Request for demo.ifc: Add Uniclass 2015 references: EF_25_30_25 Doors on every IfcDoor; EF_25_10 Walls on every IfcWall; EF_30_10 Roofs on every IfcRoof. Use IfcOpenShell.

First a look at what the model holds.

```python
import ifcopenshell

model = ifcopenshell.open("demo.ifc")
print(model.schema)
print("classifications:", [c.Name for c in model.by_type("IfcClassification")])
for ifc_class in ("IfcDoor", "IfcRoof", "IfcStair", "IfcWall", "IfcWindow"):
    print(ifc_class, len(model.by_type(ifc_class)))
```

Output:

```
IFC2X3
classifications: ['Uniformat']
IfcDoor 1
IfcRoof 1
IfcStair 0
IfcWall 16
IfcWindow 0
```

```python
import ifcopenshell
import ifcopenshell.api.classification

model = ifcopenshell.open("demo.ifc")

# IFC2X3 requires Source and Edition and has no link from the project to the system.
system = model.create_entity("IfcClassification", Source="NBS", Edition="2015", Name="Uniclass 2015")

codes = {
    "IfcDoor": ("EF_25_30_25", "Doors"),
    "IfcWall": ("EF_25_10", "Walls"),
    "IfcRoof": ("EF_30_10", "Roofs"),
}
for ifc_class, (code, name) in codes.items():
    products = model.by_type(ifc_class)
    ifcopenshell.api.classification.add_reference(
        model, products=products, classification=system, identification=code, name=name
    )
    print(code, len(products))

model.write("demo-out.ifc")
```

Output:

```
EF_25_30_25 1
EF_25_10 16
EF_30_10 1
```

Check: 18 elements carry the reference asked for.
